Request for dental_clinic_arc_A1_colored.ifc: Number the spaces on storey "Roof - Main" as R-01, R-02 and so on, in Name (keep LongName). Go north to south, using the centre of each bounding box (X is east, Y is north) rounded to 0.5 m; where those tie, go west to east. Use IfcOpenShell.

First a look at what the model holds.

```python
import ifcopenshell
import ifcopenshell.util.element
import ifcopenshell.util.placement

model = ifcopenshell.open("dental_clinic_arc_A1_colored.ifc")
print(model.schema)
storey = next(s for s in model.by_type("IfcBuildingStorey") if s.Name == "Roof - Main")
spaces = [e for e in ifcopenshell.util.element.get_decomposition(storey) if e.is_a("IfcSpace")]
for e in sorted(spaces, key=lambda e: e.id()):
    origin = ifcopenshell.util.placement.get_local_placement(e.ObjectPlacement)[:3, 3]
    print(e.id(), e.Name, e.LongName, origin.round(2) + 0.0, sep=" | ")
```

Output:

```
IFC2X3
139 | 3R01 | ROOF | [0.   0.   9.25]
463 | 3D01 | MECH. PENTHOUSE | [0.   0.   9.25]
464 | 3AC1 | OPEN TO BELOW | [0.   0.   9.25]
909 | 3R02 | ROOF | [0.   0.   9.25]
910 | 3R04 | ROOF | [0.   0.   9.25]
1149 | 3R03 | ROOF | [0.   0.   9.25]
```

```python
import ifcopenshell
import ifcopenshell.geom
import ifcopenshell.util.element
import ifcopenshell.util.shape

model = ifcopenshell.open("dental_clinic_arc_A1_colored.ifc")
settings = ifcopenshell.geom.settings()
settings.set("use-world-coords", True)


def centre(element):
    shape = ifcopenshell.geom.create_shape(settings, element)
    return ifcopenshell.util.shape.get_bbox_centroid(shape.geometry)


storey = next(s for s in model.by_type("IfcBuildingStorey") if s.Name == "Roof - Main")
spaces = [e for e in ifcopenshell.util.element.get_decomposition(storey) if e.is_a("IfcSpace")]

# Insertion points can sit at a corner or the storey origin, so sort by the geometry (in metres).
centres = {e: centre(e) for e in spaces}
spaces.sort(key=lambda e: (-round(centres[e][1] / 0.5), centres[e][0]))

for i, e in enumerate(spaces, start=1):
    number = f"R-{i:02d}"
    e.Name = number
    print(e.id(), number)

model.write("dental_clinic_arc_A1_colored-out.ifc")
```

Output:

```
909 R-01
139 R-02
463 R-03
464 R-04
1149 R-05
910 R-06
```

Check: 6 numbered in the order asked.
